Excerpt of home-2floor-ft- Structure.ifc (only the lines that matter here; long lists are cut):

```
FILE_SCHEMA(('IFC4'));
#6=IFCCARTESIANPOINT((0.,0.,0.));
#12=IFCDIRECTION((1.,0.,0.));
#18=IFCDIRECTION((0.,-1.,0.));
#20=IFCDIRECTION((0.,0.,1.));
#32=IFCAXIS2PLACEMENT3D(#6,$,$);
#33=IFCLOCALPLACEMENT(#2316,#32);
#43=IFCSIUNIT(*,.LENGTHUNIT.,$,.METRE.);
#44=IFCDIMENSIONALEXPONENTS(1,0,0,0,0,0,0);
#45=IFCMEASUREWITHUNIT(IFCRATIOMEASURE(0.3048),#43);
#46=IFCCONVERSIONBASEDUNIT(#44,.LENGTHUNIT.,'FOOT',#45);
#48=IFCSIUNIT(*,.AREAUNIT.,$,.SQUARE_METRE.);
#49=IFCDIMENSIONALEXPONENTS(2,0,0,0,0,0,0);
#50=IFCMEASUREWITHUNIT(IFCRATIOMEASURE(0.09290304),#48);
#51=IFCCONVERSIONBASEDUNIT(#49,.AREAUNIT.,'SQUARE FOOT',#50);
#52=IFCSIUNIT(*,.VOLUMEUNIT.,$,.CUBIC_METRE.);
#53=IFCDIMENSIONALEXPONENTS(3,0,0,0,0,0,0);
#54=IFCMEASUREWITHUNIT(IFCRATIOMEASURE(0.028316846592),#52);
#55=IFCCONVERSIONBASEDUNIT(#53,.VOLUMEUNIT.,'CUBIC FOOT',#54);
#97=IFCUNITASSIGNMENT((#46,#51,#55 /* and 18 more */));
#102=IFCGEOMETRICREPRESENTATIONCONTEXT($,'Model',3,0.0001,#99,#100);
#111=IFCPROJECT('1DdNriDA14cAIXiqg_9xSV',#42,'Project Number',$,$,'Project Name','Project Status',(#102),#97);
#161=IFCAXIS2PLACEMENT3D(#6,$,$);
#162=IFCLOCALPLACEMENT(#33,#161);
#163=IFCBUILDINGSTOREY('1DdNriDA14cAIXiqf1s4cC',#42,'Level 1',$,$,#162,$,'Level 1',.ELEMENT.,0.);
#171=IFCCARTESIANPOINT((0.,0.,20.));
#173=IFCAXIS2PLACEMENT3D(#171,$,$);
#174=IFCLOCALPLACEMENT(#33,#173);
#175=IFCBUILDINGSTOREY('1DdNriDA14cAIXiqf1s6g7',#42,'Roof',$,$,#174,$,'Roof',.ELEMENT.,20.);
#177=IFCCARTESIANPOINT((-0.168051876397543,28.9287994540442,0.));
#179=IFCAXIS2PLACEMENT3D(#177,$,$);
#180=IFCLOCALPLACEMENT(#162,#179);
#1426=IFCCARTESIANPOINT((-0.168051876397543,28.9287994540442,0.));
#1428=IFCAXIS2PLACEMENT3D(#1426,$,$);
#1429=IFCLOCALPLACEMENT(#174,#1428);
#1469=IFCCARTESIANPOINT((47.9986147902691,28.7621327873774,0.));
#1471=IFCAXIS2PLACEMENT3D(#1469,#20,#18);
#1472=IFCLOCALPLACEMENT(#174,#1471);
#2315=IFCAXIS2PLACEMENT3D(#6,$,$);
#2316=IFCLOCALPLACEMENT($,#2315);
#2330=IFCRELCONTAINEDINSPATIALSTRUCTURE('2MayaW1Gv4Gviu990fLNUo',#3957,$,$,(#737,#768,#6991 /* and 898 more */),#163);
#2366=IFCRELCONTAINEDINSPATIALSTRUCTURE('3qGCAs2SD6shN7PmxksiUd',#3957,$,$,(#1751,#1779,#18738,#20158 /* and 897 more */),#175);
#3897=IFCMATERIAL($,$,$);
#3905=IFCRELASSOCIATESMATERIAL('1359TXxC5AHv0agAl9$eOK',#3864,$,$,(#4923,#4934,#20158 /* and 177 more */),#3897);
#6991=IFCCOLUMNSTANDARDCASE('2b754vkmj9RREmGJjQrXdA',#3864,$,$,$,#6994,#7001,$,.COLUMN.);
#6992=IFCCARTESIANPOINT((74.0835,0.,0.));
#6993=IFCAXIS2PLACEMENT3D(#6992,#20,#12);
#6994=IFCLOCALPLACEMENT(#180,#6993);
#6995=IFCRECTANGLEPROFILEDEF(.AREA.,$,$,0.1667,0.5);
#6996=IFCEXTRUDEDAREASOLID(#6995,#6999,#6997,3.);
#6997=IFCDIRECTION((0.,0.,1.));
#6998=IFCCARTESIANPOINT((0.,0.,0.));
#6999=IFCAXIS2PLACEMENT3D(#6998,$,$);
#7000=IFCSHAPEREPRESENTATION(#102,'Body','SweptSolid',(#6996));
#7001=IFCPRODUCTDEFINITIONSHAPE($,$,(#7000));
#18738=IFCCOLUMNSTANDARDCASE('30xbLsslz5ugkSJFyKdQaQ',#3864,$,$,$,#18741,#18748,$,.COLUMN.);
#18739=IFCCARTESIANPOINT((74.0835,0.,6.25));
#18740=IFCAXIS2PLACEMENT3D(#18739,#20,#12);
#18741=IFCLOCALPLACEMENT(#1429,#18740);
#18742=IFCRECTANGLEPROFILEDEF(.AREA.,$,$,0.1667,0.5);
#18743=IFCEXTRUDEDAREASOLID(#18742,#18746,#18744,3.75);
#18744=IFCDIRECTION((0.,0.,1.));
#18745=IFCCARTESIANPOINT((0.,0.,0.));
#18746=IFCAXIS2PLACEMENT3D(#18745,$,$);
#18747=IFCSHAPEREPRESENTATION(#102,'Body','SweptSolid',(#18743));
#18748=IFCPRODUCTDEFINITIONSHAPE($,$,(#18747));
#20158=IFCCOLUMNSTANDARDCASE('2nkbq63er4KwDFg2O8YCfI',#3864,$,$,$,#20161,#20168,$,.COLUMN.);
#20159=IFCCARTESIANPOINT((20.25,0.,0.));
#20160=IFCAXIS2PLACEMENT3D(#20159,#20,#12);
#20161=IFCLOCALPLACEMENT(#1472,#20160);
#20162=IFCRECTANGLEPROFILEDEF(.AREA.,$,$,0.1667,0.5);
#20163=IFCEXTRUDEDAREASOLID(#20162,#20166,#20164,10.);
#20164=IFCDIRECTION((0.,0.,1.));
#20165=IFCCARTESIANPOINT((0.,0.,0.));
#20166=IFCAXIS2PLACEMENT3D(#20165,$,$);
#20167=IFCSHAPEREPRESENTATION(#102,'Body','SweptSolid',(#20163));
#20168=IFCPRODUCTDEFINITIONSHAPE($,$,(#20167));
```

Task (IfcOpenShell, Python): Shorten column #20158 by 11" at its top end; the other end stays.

```python
import ifcopenshell
import ifcopenshell.util.unit

model = ifcopenshell.open("home-2floor-ft- Structure.ifc")
unit_scale = ifcopenshell.util.unit.calculate_unit_scale(model)

member = model.by_id(20158)
change = -11 * 0.0254 / unit_scale

# The extrusion runs towards the end named, so only its depth changes.
body = next(r for r in member.Representation.Representations if r.RepresentationIdentifier == "Body")
solid = body.Items[0]
old_length = solid.Depth
solid.Depth += change

print(f"length {old_length:g} -> {solid.Depth:g}")

model.write("home-2floor-ft- Structure_updated.ifc")
```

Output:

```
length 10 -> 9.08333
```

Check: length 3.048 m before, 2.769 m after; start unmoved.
